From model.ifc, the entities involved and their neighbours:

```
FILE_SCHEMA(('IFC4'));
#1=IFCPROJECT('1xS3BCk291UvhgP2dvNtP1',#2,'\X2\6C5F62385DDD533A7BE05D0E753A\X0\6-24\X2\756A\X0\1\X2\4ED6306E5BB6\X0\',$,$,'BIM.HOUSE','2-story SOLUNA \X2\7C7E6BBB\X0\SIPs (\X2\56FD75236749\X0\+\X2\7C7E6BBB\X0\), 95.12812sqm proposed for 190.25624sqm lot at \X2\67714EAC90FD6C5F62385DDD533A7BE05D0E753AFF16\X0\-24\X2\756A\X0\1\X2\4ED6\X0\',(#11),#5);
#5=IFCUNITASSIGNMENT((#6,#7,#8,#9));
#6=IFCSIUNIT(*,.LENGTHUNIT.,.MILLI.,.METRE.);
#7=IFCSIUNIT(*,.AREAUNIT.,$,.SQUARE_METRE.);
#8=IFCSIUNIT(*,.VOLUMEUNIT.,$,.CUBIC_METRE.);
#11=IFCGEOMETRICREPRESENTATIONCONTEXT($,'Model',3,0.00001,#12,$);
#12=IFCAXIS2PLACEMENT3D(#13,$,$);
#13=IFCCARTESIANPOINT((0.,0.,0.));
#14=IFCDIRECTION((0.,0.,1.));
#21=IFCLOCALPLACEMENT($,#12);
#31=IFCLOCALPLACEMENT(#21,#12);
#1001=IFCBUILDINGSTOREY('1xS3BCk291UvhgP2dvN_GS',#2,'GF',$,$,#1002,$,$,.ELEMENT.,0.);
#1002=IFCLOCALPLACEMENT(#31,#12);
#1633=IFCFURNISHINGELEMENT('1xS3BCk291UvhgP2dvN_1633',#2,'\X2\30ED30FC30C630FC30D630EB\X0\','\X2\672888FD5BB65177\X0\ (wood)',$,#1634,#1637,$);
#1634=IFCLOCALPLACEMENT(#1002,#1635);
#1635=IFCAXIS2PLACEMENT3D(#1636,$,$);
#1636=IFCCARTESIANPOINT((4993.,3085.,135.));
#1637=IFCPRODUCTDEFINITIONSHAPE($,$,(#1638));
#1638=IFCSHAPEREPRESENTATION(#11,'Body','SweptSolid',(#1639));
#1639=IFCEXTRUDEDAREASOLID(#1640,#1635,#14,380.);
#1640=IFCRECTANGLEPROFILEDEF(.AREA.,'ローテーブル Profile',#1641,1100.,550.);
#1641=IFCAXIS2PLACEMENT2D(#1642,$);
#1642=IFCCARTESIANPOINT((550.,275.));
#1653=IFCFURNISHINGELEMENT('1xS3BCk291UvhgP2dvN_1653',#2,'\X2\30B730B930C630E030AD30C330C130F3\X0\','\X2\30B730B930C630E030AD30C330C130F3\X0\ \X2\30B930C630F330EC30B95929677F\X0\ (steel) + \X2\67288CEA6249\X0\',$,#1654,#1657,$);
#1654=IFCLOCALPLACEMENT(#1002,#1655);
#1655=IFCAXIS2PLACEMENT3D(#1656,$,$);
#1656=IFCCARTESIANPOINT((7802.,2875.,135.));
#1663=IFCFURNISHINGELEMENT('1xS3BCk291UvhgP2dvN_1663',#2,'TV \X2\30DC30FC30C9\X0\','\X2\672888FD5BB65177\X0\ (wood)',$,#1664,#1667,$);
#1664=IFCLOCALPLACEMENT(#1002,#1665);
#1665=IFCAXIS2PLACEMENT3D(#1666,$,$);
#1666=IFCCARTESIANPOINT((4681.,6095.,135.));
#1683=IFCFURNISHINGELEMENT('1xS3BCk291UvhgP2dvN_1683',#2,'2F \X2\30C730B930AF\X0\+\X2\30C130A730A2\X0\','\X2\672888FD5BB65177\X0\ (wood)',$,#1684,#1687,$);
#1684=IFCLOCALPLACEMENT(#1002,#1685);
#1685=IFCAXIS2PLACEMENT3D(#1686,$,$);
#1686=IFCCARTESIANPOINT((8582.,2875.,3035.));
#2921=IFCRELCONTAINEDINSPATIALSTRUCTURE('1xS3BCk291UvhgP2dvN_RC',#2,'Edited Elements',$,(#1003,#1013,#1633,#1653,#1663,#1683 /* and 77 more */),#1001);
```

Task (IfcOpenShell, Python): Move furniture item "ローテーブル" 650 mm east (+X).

```python
import ifcopenshell
import ifcopenshell.api.geometry
import ifcopenshell.util.placement
import ifcopenshell.util.unit

model = ifcopenshell.open("model.ifc")
unit_scale = ifcopenshell.util.unit.calculate_unit_scale(model)

item = model.by_guid("1xS3BCk291UvhgP2dvN_1633")
matrix = ifcopenshell.util.placement.get_local_placement(item.ObjectPlacement)
matrix[0, 3] += 0.65 / unit_scale
ifcopenshell.api.geometry.edit_object_placement(model, product=item, matrix=matrix, is_si=False)

print(ifcopenshell.util.placement.get_local_placement(item.ObjectPlacement).round(3) + 0.0)

model.write("model-out.ifc")
```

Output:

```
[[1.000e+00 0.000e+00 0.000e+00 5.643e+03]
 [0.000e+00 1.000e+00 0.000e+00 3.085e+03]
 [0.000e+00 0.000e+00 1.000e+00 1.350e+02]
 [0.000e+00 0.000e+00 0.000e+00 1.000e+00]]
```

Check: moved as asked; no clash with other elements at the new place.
